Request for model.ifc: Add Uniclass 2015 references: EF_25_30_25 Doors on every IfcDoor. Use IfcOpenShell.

First a look at what the model holds.

```python
import ifcopenshell

model = ifcopenshell.open("model.ifc")
print(model.schema)
print("classifications:", [c.Name for c in model.by_type("IfcClassification")])
for ifc_class in ("IfcDoor", "IfcRoof", "IfcStair", "IfcWall", "IfcWindow"):
    print(ifc_class, len(model.by_type(ifc_class)))
```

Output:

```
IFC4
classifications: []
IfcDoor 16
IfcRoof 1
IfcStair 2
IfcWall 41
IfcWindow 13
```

```python
import ifcopenshell
import ifcopenshell.api.classification

model = ifcopenshell.open("model.ifc")

system = ifcopenshell.api.classification.add_classification(model, classification="Uniclass 2015")

codes = {
    "IfcDoor": ("EF_25_30_25", "Doors"),
}
for ifc_class, (code, name) in codes.items():
    products = model.by_type(ifc_class)
    ifcopenshell.api.classification.add_reference(
        model, products=products, classification=system, identification=code, name=name
    )
    print(code, len(products))

model.write("model_v2.ifc")
```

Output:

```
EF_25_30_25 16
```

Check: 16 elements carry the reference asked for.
